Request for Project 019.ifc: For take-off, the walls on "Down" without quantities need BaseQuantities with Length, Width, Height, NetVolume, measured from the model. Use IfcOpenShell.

First a look at what the model holds.

```python
import ifcopenshell
import ifcopenshell.util.element
import ifcopenshell.util.unit

model = ifcopenshell.open("Project 019.ifc")
print(model.schema)
for unit_type in ("LENGTHUNIT", "AREAUNIT", "VOLUMEUNIT"):
    print(unit_type, ifcopenshell.util.unit.calculate_unit_scale(model, unit_type))
storey = next(s for s in model.by_type("IfcBuildingStorey") if s.Name == "Down")
walls = [e for e in ifcopenshell.util.element.get_decomposition(storey) if e.is_a("IfcWall")]
for e in sorted(walls, key=lambda e: e.id()):
    print(e.id(), e.is_a(), e.Name, list(ifcopenshell.util.element.get_psets(e, qtos_only=True)), sep=" | ")
```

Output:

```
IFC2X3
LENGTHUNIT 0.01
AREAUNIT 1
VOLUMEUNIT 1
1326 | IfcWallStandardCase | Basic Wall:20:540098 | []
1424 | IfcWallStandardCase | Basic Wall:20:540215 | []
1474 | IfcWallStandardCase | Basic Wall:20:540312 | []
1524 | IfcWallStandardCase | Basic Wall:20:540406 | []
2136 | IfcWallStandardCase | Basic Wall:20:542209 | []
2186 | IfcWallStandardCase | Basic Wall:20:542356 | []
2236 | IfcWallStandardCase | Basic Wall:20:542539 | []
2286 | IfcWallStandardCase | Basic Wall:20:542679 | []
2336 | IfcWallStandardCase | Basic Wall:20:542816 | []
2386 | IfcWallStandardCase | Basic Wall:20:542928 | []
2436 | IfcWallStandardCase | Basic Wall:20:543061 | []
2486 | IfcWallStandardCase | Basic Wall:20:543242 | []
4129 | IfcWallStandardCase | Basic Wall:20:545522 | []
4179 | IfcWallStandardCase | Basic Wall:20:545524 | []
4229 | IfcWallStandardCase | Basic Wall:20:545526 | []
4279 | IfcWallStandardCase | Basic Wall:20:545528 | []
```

```python
import ifcopenshell
import ifcopenshell.api.pset
import ifcopenshell.geom
import ifcopenshell.util.element
import ifcopenshell.util.shape
import ifcopenshell.util.unit

model = ifcopenshell.open("Project 019.ifc")
unit_scale = ifcopenshell.util.unit.calculate_unit_scale(model)
volume_scale = ifcopenshell.util.unit.calculate_unit_scale(model, "VOLUMEUNIT")
settings = ifcopenshell.geom.settings()

storey = next(s for s in model.by_type("IfcBuildingStorey") if s.Name == "Down")
walls = [e for e in ifcopenshell.util.element.get_decomposition(storey) if e.is_a("IfcWall")]

for e in sorted(walls, key=lambda e: e.id()):
    if ifcopenshell.util.element.get_psets(e, qtos_only=True, should_inherit=False):
        continue
    # Geometry comes back in metres, in the element's own axes.
    shape = ifcopenshell.geom.create_shape(settings, e)
    values = {
        "Length": ifcopenshell.util.shape.get_x(shape.geometry) / unit_scale,
        "Width": ifcopenshell.util.shape.get_y(shape.geometry) / unit_scale,
        "Height": ifcopenshell.util.shape.get_z(shape.geometry) / unit_scale,
        "NetVolume": ifcopenshell.util.shape.get_volume(shape.geometry) / volume_scale,
    }
    qto = ifcopenshell.api.pset.add_qto(model, product=e, name="BaseQuantities")
    ifcopenshell.api.pset.edit_qto(model, qto=qto, properties=values)
    print(e.id(), {k: round(v, 3) for k, v in values.items()})

model.write("Project 019_v2.ifc")
```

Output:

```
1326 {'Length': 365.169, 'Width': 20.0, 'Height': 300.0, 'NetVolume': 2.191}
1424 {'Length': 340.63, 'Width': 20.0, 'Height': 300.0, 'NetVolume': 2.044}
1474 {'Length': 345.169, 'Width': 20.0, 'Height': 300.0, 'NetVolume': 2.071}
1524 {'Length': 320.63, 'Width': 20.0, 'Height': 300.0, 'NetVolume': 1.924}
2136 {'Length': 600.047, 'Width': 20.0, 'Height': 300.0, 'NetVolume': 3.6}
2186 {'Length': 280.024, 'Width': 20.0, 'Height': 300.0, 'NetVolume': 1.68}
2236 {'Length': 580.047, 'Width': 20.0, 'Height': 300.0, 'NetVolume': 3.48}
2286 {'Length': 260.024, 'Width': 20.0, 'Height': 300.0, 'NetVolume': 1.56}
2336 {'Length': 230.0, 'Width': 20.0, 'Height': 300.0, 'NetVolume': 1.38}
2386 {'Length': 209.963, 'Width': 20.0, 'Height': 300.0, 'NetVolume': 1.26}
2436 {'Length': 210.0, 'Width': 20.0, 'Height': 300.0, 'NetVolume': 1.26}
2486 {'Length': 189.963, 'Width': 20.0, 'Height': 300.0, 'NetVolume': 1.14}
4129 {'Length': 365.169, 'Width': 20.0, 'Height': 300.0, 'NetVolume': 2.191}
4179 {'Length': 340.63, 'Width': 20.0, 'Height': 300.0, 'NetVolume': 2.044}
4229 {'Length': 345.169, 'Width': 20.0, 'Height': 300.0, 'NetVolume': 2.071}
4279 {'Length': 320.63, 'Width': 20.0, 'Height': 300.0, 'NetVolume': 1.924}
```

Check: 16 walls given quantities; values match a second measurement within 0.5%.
